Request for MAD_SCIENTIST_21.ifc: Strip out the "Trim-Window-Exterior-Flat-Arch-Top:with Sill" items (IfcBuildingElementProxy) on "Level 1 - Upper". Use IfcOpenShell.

First a look at what the model holds.

```python
import ifcopenshell
import ifcopenshell.util.element

model = ifcopenshell.open("MAD_SCIENTIST_21.ifc")
print(model.schema)
storey = next(s for s in model.by_type("IfcBuildingStorey") if s.Name == "Level 1 - Upper")
proxies = [e for e in ifcopenshell.util.element.get_decomposition(storey) if e.is_a("IfcBuildingElementProxy")]
seen = {}
for e in proxies:
    element_type = ifcopenshell.util.element.get_type(e)
    name = element_type.Name if element_type not in (None, e) else None
    seen[name] = seen.get(name, 0) + 1
for name, count in sorted(seen.items(), key=str):
    print(count, "x", name)
```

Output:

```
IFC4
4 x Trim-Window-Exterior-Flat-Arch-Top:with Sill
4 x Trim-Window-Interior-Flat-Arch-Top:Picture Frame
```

```python
import ifcopenshell
import ifcopenshell.api.root
import ifcopenshell.util.element

model = ifcopenshell.open("MAD_SCIENTIST_21.ifc")

storey = next(s for s in model.by_type("IfcBuildingStorey") if s.Name == "Level 1 - Upper")
proxies = [e for e in ifcopenshell.util.element.get_decomposition(storey) if e.is_a("IfcBuildingElementProxy")]
targets = [e for e in proxies if (t := ifcopenshell.util.element.get_type(e)) not in (None, e) and t.Name == "Trim-Window-Exterior-Flat-Arch-Top:with Sill"]

for e in targets:
    ifcopenshell.api.root.remove_product(model, product=e)
print(len(targets), "removed")

model.write("MAD_SCIENTIST_21_rev.ifc")
```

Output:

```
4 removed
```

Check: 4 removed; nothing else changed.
